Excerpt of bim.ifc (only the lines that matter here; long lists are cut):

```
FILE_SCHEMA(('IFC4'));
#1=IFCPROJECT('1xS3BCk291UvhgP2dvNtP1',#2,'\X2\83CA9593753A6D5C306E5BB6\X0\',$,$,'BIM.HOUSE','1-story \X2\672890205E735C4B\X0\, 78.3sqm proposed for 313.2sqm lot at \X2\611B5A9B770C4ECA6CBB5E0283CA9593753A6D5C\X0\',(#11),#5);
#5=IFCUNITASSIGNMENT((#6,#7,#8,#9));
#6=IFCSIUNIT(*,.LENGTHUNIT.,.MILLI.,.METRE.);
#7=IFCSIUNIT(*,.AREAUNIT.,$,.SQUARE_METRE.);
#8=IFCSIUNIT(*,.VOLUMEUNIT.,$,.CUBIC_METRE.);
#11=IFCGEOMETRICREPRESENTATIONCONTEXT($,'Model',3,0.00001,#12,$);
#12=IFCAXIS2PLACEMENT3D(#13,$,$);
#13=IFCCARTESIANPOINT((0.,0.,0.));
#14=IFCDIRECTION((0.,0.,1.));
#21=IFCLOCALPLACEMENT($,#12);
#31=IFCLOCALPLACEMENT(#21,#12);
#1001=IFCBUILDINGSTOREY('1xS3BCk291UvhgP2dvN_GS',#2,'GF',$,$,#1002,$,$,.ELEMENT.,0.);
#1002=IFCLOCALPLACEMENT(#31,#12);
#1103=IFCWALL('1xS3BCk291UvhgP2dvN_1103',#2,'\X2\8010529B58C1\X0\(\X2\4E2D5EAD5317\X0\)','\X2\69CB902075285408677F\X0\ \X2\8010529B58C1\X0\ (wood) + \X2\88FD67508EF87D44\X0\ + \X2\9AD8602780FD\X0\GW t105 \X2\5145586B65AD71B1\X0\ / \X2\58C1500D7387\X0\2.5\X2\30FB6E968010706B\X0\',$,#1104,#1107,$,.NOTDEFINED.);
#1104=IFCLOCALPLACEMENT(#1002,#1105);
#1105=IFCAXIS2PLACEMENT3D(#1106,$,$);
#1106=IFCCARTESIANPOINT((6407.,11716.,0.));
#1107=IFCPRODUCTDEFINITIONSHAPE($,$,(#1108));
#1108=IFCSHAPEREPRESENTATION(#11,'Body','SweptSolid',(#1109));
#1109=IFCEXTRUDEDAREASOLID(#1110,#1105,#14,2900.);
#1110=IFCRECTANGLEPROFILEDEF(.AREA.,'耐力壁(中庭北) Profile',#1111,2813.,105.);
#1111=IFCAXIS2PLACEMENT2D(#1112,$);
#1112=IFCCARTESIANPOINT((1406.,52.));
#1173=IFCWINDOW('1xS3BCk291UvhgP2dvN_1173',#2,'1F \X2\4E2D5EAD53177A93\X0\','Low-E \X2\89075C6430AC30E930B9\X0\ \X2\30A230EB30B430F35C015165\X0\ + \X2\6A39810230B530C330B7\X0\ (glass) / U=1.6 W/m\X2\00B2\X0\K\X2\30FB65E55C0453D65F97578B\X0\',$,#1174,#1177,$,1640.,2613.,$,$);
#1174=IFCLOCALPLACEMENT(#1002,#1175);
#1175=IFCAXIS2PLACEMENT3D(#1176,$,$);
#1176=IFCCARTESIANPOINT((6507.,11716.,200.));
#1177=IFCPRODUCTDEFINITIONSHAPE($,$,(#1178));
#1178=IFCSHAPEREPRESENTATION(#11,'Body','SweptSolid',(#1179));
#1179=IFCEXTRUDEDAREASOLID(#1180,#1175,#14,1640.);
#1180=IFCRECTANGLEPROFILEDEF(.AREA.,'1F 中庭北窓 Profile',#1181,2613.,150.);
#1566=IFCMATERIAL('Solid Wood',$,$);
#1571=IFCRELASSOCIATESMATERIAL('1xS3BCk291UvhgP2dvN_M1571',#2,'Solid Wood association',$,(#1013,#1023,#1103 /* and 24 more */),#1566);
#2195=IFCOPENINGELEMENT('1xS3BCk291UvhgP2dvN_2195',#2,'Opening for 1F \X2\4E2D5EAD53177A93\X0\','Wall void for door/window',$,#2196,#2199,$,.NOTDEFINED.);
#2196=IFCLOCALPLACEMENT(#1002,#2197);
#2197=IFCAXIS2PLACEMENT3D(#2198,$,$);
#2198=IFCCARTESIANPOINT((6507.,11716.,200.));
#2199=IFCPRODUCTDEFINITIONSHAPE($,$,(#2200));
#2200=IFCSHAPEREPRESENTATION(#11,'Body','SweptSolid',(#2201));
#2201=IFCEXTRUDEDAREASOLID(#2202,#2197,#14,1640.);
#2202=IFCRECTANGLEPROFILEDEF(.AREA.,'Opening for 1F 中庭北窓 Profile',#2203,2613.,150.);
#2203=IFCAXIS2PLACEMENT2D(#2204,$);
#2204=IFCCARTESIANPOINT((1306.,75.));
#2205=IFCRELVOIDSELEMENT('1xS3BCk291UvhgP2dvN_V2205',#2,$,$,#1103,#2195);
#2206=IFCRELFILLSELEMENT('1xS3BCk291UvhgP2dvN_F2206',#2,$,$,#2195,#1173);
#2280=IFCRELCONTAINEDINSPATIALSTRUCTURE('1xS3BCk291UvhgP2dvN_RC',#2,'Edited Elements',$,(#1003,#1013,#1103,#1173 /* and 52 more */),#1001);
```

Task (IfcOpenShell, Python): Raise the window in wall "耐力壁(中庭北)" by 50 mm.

```python
import numpy as np
import ifcopenshell
import ifcopenshell.api.geometry
import ifcopenshell.util.placement
import ifcopenshell.util.unit

model = ifcopenshell.open("bim.ifc")
unit_scale = ifcopenshell.util.unit.calculate_unit_scale(model)

window = model.by_guid("1xS3BCk291UvhgP2dvN_1173")
opening = window.FillsVoids[0].RelatingOpeningElement
dz = 50.0

shift = np.array([0.0, 0.0, dz])
# The window is not placed relative to its opening, so move both.
for product in (opening, window):
    matrix = ifcopenshell.util.placement.get_local_placement(product.ObjectPlacement)
    matrix[:3, 3] += shift
    ifcopenshell.api.geometry.edit_object_placement(model, product=product, matrix=matrix, is_si=False)

print(f"moved by {dz * unit_scale:+.3f} m")

model.write("bim_rev.ifc")
```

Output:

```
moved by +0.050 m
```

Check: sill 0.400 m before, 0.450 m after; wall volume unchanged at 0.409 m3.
